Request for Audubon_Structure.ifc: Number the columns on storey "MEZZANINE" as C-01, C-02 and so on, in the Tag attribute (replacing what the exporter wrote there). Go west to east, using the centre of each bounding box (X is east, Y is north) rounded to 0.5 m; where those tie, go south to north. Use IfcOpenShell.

First a look at what the model holds.

```python
import ifcopenshell
import ifcopenshell.util.element
import ifcopenshell.util.placement

model = ifcopenshell.open("Audubon_Structure.ifc")
print(model.schema)
storey = next(s for s in model.by_type("IfcBuildingStorey") if s.Name == "MEZZANINE")
columns = [e for e in ifcopenshell.util.element.get_decomposition(storey) if e.is_a("IfcColumn")]
for e in sorted(columns, key=lambda e: e.id()):
    origin = ifcopenshell.util.placement.get_local_placement(e.ObjectPlacement)[:3, 3]
    print(e.id(), e.Tag, e.Name, origin.round(2) + 0.0, sep=" | ")
```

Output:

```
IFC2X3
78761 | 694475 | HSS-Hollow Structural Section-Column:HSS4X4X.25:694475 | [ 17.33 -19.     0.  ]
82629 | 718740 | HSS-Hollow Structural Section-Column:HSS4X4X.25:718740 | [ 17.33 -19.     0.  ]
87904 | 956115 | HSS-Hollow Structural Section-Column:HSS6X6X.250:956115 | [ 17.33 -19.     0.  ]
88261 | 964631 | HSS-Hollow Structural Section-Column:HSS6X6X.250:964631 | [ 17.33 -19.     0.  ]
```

```python
import ifcopenshell
import ifcopenshell.geom
import ifcopenshell.util.element
import ifcopenshell.util.shape

model = ifcopenshell.open("Audubon_Structure.ifc")
settings = ifcopenshell.geom.settings()
settings.set("use-world-coords", True)


def centre(element):
    shape = ifcopenshell.geom.create_shape(settings, element)
    return ifcopenshell.util.shape.get_bbox_centroid(shape.geometry)


storey = next(s for s in model.by_type("IfcBuildingStorey") if s.Name == "MEZZANINE")
columns = [e for e in ifcopenshell.util.element.get_decomposition(storey) if e.is_a("IfcColumn")]

# Insertion points can sit at a corner or the storey origin, so sort by the geometry (in metres).
centres = {e: centre(e) for e in columns}
columns.sort(key=lambda e: (round(centres[e][0] / 0.5), centres[e][1]))

for i, e in enumerate(columns, start=1):
    number = f"C-{i:02d}"
    e.Tag = number
    print(e.id(), number)

model.write("Audubon_Structure_v2.ifc")
```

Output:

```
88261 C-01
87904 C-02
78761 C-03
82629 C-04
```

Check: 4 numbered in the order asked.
